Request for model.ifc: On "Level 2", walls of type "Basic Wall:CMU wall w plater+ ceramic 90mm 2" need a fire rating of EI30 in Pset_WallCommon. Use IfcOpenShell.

First a look at what the model holds.

```python
import ifcopenshell
import ifcopenshell.util.element

model = ifcopenshell.open("model.ifc")
print(model.schema)
storey = next(s for s in model.by_type("IfcBuildingStorey") if s.Name == "Level 2")
walls = [e for e in ifcopenshell.util.element.get_decomposition(storey) if e.is_a("IfcWall")]
seen = {}
for e in walls:
    element_type = ifcopenshell.util.element.get_type(e)
    key = (element_type.Name if element_type != e and element_type else None, ifcopenshell.util.element.get_pset(e, "Pset_WallCommon", "FireRating"))
    seen[key] = seen.get(key, 0) + 1
for (name, value), count in sorted(seen.items(), key=str):
    print(count, "x", name, "|", value)
```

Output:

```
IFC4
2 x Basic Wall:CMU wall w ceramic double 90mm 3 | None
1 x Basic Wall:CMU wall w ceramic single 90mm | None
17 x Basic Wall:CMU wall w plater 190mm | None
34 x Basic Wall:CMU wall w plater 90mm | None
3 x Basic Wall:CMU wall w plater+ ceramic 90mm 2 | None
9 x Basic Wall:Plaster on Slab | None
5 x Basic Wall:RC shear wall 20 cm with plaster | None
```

```python
import ifcopenshell
import ifcopenshell.api.pset
import ifcopenshell.util.element

model = ifcopenshell.open("model.ifc")

storey = next(s for s in model.by_type("IfcBuildingStorey") if s.Name == "Level 2")
walls = [e for e in ifcopenshell.util.element.get_decomposition(storey) if e.is_a("IfcWall")]

count = 0
for e in walls:
    element_type = ifcopenshell.util.element.get_type(e)
    if element_type in (None, e) or element_type.Name != "Basic Wall:CMU wall w plater+ ceramic 90mm 2":
        continue
    # add_pset returns the element's existing set when there is one.
    pset = ifcopenshell.api.pset.add_pset(model, product=e, name="Pset_WallCommon")
    ifcopenshell.api.pset.edit_pset(model, pset=pset, properties={"FireRating": "EI30"})
    count += 1

print(count, "walls updated")

model.write("model_rev.ifc")
```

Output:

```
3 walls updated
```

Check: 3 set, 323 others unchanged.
